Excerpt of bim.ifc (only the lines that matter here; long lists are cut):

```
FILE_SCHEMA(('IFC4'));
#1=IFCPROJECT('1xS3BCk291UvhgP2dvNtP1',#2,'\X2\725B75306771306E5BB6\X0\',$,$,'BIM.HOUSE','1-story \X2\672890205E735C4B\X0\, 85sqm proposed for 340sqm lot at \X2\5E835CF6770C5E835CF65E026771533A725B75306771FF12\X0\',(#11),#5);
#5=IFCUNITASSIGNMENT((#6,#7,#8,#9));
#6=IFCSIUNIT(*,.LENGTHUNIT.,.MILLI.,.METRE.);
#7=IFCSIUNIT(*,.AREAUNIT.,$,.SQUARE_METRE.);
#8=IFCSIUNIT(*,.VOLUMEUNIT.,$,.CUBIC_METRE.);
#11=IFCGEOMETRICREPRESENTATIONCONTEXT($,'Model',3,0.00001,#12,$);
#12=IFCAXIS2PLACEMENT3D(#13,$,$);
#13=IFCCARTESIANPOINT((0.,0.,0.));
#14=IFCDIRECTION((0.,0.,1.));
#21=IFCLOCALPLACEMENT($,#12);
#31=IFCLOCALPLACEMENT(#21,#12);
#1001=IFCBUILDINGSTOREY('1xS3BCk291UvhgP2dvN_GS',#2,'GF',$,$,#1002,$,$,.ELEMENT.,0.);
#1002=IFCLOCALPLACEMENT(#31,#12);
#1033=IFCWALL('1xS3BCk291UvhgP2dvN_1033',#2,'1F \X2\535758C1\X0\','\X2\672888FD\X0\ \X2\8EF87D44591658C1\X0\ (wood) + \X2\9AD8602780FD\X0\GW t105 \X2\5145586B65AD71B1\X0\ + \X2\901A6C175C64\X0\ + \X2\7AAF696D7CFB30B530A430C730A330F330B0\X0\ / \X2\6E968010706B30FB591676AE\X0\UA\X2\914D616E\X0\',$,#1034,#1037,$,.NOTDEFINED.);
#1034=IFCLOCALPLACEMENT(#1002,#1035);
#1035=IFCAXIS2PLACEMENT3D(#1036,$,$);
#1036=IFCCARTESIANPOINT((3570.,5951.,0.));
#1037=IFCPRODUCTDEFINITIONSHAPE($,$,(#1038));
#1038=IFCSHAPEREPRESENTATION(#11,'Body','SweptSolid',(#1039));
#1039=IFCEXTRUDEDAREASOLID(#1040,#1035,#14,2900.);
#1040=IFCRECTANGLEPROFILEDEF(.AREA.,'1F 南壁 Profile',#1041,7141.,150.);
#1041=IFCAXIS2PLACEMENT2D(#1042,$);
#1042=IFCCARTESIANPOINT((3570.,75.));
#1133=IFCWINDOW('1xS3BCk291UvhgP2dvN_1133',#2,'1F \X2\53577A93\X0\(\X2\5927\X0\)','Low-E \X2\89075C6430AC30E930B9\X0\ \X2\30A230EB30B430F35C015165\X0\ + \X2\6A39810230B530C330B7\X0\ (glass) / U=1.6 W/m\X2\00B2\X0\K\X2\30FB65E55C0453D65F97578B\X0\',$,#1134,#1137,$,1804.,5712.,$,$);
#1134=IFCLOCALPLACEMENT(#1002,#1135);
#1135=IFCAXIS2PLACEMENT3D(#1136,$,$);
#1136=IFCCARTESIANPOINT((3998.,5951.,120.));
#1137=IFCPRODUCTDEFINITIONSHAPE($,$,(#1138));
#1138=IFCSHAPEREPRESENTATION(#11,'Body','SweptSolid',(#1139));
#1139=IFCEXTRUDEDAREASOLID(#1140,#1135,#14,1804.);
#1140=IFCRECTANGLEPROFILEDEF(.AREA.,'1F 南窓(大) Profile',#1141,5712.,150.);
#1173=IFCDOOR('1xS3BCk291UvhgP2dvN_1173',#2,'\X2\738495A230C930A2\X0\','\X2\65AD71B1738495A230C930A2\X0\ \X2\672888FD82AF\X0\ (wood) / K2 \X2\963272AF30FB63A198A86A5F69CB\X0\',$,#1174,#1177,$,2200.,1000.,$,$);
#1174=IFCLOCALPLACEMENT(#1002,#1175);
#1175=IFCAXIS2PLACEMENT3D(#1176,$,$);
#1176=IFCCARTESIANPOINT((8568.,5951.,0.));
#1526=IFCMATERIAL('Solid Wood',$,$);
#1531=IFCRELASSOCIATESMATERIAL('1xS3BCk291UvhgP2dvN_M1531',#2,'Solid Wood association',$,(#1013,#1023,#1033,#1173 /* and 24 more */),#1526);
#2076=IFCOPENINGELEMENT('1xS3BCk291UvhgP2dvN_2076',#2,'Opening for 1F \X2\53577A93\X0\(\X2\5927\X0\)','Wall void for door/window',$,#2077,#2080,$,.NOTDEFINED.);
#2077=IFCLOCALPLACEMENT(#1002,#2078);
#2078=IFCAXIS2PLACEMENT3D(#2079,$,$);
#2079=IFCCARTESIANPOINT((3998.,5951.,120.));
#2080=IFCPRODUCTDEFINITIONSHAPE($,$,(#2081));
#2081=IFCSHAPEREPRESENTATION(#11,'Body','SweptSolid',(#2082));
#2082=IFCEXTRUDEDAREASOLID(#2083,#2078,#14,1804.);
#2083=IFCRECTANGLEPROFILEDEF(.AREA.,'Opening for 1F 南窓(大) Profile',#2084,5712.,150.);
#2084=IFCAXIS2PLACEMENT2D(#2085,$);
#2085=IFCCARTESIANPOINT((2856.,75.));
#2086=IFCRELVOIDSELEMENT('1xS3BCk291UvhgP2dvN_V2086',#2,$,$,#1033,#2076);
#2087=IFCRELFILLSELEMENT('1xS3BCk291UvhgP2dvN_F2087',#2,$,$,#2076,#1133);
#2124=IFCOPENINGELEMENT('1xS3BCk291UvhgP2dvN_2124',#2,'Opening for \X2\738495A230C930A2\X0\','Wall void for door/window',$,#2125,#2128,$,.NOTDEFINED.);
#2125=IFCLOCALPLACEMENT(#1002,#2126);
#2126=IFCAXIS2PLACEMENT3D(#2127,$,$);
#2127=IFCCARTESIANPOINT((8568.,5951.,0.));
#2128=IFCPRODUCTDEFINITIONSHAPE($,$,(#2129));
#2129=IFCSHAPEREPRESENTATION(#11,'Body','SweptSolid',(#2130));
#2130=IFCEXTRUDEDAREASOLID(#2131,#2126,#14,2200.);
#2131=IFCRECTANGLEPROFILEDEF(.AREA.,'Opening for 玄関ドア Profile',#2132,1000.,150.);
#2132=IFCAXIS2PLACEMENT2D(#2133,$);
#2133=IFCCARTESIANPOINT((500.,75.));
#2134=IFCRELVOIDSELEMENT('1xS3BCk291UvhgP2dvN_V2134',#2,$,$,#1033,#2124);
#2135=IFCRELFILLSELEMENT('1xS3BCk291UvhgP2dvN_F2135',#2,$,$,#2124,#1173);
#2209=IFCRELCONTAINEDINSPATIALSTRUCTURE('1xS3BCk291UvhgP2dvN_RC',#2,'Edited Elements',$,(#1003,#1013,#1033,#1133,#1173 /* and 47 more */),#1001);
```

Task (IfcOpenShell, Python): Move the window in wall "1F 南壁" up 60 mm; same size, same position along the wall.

```python
import numpy as np
import ifcopenshell
import ifcopenshell.api.geometry
import ifcopenshell.util.placement
import ifcopenshell.util.unit

model = ifcopenshell.open("bim.ifc")
unit_scale = ifcopenshell.util.unit.calculate_unit_scale(model)

window = model.by_guid("1xS3BCk291UvhgP2dvN_1133")
opening = window.FillsVoids[0].RelatingOpeningElement
dz = 0.06 / unit_scale

shift = np.array([0.0, 0.0, dz])
# The window is not placed relative to its opening, so move both.
for product in (opening, window):
    matrix = ifcopenshell.util.placement.get_local_placement(product.ObjectPlacement)
    matrix[:3, 3] += shift
    ifcopenshell.api.geometry.edit_object_placement(model, product=product, matrix=matrix, is_si=False)

print(f"moved by {dz * unit_scale:+.3f} m")

model.write("bim_updated.ifc")
```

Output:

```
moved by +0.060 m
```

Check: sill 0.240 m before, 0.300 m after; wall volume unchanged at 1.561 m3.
